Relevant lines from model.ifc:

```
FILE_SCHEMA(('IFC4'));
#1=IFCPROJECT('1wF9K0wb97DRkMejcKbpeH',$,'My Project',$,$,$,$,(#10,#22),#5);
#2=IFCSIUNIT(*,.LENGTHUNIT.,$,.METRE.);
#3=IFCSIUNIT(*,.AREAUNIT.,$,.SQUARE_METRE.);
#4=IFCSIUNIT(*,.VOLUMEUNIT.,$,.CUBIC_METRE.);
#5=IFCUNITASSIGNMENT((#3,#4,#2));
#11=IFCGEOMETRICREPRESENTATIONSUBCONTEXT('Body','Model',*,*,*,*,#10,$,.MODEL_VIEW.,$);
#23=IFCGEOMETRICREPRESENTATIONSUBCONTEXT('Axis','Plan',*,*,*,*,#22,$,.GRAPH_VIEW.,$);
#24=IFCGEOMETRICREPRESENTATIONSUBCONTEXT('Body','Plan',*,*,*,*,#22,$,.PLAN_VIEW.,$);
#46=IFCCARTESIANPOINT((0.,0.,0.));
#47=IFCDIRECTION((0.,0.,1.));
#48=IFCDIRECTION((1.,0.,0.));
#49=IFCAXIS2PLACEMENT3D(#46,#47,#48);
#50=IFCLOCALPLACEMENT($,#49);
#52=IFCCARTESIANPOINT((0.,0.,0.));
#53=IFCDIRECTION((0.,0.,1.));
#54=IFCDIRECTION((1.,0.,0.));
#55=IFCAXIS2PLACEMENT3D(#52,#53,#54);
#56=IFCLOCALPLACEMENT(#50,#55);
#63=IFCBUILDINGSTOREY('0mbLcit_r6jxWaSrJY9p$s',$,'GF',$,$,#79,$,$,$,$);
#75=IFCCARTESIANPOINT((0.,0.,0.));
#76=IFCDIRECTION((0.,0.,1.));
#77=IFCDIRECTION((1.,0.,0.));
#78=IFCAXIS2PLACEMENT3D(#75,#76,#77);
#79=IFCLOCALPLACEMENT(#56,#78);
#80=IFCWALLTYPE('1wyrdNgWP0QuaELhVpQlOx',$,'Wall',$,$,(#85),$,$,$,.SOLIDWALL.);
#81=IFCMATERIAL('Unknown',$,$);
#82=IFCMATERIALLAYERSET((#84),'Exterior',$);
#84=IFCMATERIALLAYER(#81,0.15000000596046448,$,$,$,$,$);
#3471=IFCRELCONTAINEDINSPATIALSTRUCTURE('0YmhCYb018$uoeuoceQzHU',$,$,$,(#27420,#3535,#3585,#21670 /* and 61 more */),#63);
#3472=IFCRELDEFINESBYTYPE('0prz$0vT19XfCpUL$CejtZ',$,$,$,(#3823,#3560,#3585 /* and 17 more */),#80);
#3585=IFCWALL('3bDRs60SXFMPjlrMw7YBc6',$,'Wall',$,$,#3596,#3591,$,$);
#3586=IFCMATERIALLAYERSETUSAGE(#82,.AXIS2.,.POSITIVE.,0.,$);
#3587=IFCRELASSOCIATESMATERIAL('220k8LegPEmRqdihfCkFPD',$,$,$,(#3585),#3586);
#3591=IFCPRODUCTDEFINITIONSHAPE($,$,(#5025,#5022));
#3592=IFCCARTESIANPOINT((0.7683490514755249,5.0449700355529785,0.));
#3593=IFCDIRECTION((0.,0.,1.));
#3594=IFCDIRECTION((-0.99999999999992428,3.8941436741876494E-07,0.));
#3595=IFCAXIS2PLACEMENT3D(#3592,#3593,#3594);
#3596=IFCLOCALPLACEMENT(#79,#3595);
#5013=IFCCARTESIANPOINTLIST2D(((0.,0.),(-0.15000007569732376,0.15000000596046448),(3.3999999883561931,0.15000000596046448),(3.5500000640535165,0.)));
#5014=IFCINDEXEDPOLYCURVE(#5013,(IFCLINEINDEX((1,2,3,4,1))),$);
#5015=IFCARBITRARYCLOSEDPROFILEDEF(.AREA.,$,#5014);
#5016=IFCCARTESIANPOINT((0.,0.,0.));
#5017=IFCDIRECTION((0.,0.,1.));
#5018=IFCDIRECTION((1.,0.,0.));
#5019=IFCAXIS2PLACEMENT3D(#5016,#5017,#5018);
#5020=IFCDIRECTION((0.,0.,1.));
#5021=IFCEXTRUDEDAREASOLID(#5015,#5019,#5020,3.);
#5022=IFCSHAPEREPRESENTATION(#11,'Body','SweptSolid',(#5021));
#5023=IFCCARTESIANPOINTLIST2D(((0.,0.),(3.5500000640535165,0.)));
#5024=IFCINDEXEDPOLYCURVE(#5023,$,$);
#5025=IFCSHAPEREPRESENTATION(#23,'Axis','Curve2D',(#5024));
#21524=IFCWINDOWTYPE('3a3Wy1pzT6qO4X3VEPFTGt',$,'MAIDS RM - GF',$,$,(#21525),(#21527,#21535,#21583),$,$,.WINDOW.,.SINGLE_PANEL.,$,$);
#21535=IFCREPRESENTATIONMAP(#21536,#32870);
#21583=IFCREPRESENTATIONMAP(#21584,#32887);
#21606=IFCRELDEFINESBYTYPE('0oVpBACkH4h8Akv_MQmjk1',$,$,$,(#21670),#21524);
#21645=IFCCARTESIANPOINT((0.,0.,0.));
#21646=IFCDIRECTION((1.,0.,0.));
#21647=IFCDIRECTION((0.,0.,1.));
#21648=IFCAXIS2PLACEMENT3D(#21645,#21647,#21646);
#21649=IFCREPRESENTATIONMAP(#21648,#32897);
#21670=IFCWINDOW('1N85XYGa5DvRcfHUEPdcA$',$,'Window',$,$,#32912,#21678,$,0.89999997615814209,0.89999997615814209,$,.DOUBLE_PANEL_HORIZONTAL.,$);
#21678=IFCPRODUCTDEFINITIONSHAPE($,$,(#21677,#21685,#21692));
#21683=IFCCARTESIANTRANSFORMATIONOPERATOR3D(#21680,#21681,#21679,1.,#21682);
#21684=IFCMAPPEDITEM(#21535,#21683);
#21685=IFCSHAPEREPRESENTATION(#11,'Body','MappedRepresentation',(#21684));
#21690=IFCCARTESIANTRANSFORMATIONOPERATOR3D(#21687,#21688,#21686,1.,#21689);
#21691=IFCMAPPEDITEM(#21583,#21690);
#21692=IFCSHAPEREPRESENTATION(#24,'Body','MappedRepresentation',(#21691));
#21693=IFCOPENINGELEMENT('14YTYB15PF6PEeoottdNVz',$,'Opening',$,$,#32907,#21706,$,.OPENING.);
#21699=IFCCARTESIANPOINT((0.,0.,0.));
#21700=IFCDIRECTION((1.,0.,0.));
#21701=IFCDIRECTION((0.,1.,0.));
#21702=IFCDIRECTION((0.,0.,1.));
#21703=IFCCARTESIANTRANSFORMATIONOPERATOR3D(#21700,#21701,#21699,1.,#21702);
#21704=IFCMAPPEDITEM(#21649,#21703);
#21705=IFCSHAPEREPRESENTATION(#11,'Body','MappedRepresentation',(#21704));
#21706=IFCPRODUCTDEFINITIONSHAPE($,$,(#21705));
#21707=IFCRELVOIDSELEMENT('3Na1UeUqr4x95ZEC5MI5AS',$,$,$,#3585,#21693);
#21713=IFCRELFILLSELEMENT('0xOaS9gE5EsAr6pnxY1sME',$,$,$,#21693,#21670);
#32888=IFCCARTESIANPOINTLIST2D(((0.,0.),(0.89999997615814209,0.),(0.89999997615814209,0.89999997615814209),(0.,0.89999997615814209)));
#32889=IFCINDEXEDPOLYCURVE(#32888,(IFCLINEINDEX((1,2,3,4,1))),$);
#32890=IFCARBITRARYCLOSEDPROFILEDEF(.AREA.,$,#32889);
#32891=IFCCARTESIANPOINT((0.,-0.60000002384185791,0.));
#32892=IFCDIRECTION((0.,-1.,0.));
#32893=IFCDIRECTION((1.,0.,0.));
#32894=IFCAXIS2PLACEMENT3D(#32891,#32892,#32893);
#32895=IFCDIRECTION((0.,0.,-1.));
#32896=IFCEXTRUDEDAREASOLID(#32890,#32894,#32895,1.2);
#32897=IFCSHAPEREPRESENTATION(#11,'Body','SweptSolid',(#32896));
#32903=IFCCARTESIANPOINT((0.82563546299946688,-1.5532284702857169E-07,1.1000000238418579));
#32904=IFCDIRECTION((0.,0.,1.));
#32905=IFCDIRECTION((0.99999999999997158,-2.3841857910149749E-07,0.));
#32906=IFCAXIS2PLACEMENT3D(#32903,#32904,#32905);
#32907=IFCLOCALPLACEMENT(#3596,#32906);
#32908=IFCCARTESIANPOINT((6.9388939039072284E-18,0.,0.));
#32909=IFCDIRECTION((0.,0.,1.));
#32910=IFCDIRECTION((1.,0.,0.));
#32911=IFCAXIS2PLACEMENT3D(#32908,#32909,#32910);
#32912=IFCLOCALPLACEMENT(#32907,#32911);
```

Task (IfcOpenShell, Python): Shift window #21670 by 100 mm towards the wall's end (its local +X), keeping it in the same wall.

```python
import ifcopenshell
import ifcopenshell.api.geometry
import ifcopenshell.util.placement
import ifcopenshell.util.unit

model = ifcopenshell.open("model.ifc")
unit_scale = ifcopenshell.util.unit.calculate_unit_scale(model)

window = model.by_guid("1N85XYGa5DvRcfHUEPdcA$")
opening = window.FillsVoids[0].RelatingOpeningElement
wall = opening.VoidsElements[0].RelatingBuildingElement

wall_matrix = ifcopenshell.util.placement.get_local_placement(wall.ObjectPlacement)
shift = wall_matrix[:3, 0] * 0.1 / unit_scale
before = ifcopenshell.util.placement.get_local_placement(window.ObjectPlacement)[:3, 3].copy()

# The window is placed relative to its opening, so it follows when the opening moves.
matrix = ifcopenshell.util.placement.get_local_placement(opening.ObjectPlacement)
matrix[:3, 3] += shift
ifcopenshell.api.geometry.edit_object_placement(
    model, product=opening, matrix=matrix, is_si=False, should_transform_children=True
)

after = ifcopenshell.util.placement.get_local_placement(window.ObjectPlacement)[:3, 3]
print("window moved by", (after - before).round(3) + 0.0)

model.write("model_v2.ifc")
```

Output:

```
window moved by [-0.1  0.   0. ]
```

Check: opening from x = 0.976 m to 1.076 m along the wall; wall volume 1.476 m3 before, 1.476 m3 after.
